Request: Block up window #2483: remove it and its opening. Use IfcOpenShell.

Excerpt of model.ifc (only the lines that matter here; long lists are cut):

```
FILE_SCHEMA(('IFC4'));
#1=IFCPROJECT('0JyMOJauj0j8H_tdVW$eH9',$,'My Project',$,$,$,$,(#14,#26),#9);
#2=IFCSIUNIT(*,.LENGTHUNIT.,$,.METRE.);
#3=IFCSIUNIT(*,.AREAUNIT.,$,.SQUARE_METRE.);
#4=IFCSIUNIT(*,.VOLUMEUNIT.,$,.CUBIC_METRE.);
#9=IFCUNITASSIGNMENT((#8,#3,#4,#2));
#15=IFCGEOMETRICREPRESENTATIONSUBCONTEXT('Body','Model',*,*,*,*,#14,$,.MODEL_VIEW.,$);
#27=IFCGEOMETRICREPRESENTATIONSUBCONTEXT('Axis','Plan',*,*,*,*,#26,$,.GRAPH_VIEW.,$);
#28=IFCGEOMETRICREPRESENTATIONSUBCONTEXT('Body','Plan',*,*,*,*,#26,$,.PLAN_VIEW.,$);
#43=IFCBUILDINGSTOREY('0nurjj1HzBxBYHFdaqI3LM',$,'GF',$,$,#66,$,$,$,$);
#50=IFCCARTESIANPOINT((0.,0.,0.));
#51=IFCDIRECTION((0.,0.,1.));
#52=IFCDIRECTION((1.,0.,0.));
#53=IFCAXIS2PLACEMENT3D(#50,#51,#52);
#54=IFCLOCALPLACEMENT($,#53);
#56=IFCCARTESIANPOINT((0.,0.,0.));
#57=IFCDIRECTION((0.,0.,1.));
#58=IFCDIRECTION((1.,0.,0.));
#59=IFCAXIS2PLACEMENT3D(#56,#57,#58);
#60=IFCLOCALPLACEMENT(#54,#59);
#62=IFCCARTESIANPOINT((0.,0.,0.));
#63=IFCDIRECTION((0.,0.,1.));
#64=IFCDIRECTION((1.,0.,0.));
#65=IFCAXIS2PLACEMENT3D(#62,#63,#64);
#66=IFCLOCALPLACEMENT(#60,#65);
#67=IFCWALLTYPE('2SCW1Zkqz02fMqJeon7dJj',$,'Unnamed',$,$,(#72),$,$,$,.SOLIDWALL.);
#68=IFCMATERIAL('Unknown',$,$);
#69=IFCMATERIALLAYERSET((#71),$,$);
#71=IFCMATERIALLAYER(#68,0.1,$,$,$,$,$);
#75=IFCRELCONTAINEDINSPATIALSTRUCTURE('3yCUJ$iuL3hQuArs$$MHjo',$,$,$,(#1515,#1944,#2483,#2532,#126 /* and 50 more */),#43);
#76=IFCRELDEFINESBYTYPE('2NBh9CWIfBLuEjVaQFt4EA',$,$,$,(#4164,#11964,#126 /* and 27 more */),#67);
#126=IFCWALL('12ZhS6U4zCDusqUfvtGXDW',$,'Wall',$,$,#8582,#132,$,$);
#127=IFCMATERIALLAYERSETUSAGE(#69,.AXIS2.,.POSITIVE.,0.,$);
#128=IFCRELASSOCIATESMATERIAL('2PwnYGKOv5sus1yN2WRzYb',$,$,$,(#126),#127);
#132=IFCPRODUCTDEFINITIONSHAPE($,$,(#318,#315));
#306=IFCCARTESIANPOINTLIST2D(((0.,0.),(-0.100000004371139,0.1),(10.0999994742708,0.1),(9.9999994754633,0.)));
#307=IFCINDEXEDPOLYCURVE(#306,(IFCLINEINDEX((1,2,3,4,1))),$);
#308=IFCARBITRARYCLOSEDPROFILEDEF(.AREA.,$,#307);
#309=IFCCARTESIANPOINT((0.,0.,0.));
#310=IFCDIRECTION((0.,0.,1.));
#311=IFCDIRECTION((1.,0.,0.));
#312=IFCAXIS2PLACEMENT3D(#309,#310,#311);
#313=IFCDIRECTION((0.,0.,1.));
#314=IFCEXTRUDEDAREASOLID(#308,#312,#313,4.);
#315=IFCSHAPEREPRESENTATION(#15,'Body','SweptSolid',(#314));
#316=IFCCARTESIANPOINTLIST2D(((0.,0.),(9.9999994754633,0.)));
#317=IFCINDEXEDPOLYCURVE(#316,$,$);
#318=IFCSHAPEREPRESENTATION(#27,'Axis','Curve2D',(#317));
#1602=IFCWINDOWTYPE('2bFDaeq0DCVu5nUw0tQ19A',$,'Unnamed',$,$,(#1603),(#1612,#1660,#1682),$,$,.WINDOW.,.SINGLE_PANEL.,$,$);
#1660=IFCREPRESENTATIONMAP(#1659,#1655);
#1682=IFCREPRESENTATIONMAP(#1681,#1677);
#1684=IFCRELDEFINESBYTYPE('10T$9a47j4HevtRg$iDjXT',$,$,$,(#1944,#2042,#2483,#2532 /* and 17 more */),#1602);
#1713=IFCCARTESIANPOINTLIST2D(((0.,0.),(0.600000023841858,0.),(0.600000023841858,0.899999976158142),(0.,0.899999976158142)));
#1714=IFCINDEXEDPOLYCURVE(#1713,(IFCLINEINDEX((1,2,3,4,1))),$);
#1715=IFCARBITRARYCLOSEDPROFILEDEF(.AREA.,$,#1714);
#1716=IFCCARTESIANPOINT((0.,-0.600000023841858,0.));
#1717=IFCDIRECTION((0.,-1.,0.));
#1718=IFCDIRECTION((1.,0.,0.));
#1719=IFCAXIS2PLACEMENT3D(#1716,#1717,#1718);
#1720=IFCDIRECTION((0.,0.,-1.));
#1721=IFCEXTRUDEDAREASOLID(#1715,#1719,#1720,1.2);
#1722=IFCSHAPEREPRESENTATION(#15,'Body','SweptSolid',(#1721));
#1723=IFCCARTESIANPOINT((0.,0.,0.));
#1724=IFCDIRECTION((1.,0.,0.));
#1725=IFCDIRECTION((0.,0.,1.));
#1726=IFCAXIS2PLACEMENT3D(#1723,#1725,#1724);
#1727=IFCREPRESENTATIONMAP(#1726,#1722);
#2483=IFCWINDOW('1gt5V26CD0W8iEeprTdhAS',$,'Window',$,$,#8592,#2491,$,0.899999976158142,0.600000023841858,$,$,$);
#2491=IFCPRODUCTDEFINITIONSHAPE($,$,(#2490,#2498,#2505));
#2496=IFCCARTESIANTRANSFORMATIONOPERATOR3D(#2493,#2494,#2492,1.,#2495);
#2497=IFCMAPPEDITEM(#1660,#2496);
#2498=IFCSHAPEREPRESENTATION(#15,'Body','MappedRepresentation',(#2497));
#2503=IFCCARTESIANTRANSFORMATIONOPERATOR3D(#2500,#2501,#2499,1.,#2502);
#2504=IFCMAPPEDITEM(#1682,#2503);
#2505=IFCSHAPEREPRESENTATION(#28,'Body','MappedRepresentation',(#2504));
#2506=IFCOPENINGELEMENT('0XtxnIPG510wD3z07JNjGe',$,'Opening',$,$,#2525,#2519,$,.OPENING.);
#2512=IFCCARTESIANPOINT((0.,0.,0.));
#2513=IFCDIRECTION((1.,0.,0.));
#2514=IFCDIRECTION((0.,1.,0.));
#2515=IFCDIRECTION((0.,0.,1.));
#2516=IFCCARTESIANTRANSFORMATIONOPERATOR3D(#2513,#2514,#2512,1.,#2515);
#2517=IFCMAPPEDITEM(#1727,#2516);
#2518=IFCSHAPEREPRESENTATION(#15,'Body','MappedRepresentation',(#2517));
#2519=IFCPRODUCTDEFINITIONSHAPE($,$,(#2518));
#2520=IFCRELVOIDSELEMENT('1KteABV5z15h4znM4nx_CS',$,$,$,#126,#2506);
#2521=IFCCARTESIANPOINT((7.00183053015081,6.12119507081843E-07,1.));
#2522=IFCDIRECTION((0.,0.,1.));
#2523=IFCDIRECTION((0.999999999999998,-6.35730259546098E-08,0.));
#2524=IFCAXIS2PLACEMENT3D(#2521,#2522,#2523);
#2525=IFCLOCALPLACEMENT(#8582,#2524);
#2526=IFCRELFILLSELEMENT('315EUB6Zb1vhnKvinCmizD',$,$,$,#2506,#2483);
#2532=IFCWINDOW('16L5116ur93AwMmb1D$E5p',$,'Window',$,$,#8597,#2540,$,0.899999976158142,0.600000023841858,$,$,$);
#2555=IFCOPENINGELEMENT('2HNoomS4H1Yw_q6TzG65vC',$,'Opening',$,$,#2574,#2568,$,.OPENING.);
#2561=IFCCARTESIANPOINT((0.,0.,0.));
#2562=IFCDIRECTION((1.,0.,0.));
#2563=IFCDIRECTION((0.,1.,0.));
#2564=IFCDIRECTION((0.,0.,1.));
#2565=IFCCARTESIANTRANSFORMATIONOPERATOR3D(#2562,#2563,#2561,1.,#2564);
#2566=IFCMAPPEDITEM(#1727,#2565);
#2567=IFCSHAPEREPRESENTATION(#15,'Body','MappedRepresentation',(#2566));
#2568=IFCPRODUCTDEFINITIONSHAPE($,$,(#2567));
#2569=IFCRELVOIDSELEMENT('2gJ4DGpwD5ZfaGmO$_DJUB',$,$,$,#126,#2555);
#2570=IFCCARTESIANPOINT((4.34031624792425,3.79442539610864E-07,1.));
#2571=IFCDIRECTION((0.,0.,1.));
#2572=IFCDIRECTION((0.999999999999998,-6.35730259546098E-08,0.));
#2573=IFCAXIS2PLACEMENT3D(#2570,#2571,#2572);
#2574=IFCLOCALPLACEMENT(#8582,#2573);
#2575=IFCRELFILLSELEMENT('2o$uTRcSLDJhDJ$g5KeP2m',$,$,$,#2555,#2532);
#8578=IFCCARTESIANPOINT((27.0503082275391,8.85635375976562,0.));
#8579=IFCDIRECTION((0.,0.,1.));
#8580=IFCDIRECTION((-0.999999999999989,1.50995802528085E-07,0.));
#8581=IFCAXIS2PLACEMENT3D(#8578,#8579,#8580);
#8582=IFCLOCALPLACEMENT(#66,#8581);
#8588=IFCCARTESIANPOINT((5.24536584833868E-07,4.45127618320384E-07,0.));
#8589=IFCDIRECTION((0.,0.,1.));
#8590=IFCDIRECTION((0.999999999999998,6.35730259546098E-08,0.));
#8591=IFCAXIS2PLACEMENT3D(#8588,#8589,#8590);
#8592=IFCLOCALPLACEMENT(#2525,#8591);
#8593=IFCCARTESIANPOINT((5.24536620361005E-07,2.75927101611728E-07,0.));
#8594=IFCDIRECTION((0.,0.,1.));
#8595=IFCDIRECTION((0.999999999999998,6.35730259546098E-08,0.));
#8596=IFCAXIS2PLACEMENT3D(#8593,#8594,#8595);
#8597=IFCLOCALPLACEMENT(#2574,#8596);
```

```python
import ifcopenshell
import ifcopenshell.api.feature
import ifcopenshell.api.root
import ifcopenshell.geom
import ifcopenshell.util.shape

model = ifcopenshell.open("model.ifc")
settings = ifcopenshell.geom.settings()


def volume(element):
    """Net volume in cubic metres, openings subtracted."""
    shape = ifcopenshell.geom.create_shape(settings, element)
    return ifcopenshell.util.shape.get_volume(shape.geometry)


window = model.by_id(2483)
opening = window.FillsVoids[0].RelatingOpeningElement
wall = opening.VoidsElements[0].RelatingBuildingElement
before = volume(wall)

ifcopenshell.api.root.remove_product(model, product=window)
ifcopenshell.api.feature.remove_feature(model, feature=opening)

after = volume(wall)

print(f"wall volume {before:.3f} -> {after:.3f} m3")

model.write("model-out.ifc")
```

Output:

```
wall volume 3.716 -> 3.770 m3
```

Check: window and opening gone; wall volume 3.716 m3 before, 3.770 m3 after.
